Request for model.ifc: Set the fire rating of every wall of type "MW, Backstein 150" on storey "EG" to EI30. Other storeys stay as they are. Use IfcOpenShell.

First a look at what the model holds.

```python
import ifcopenshell
import ifcopenshell.util.element

model = ifcopenshell.open("model.ifc")
print(model.schema)
storey = next(s for s in model.by_type("IfcBuildingStorey") if s.Name == "EG")
walls = [e for e in ifcopenshell.util.element.get_decomposition(storey) if e.is_a("IfcWall")]
seen = {}
for e in walls:
    element_type = ifcopenshell.util.element.get_type(e)
    key = (element_type.Name if element_type != e and element_type else None, ifcopenshell.util.element.get_pset(e, "Pset_WallCommon", "FireRating"))
    seen[key] = seen.get(key, 0) + 1
for (name, value), count in sorted(seen.items(), key=str):
    print(count, "x", name, "|", value)
```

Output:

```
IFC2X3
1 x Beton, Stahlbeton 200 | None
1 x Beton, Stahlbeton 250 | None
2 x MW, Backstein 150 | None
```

```python
import ifcopenshell
import ifcopenshell.api.pset
import ifcopenshell.util.element

model = ifcopenshell.open("model.ifc")

storey = next(s for s in model.by_type("IfcBuildingStorey") if s.Name == "EG")
walls = [e for e in ifcopenshell.util.element.get_decomposition(storey) if e.is_a("IfcWall")]

count = 0
for e in walls:
    element_type = ifcopenshell.util.element.get_type(e)
    if element_type in (None, e) or element_type.Name != "MW, Backstein 150":
        continue
    # add_pset returns the element's existing set when there is one.
    pset = ifcopenshell.api.pset.add_pset(model, product=e, name="Pset_WallCommon")
    ifcopenshell.api.pset.edit_pset(model, pset=pset, properties={"FireRating": "EI30"})
    count += 1

print(count, "walls updated")

model.write("model-out.ifc")
```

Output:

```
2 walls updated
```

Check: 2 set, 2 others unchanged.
